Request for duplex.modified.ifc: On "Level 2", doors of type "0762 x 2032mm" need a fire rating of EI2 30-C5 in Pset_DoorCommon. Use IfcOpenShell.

First a look at what the model holds.

```python
import ifcopenshell
import ifcopenshell.util.element

model = ifcopenshell.open("duplex.modified.ifc")
print(model.schema)
storey = next(s for s in model.by_type("IfcBuildingStorey") if s.Name == "Level 2")
doors = [e for e in ifcopenshell.util.element.get_decomposition(storey) if e.is_a("IfcDoor")]
seen = {}
for e in doors:
    element_type = ifcopenshell.util.element.get_type(e)
    key = (element_type.Name if element_type != e and element_type else None, ifcopenshell.util.element.get_pset(e, "Pset_DoorCommon", "FireRating"))
    seen[key] = seen.get(key, 0) + 1
for (name, value), count in sorted(seen.items(), key=str):
    print(count, "x", name, "|", value)
```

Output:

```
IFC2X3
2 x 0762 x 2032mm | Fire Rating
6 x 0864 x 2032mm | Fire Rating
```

```python
import ifcopenshell
import ifcopenshell.api.pset
import ifcopenshell.util.element

model = ifcopenshell.open("duplex.modified.ifc")

storey = next(s for s in model.by_type("IfcBuildingStorey") if s.Name == "Level 2")
doors = [e for e in ifcopenshell.util.element.get_decomposition(storey) if e.is_a("IfcDoor")]

count = 0
for e in doors:
    element_type = ifcopenshell.util.element.get_type(e)
    if element_type in (None, e) or element_type.Name != "0762 x 2032mm":
        continue
    # add_pset returns the element's existing set when there is one.
    pset = ifcopenshell.api.pset.add_pset(model, product=e, name="Pset_DoorCommon")
    ifcopenshell.api.pset.edit_pset(model, pset=pset, properties={"FireRating": "EI2 30-C5"})
    count += 1

print(count, "doors updated")

model.write("duplex.modified_v2.ifc")
```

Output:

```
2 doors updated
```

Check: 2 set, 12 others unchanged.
